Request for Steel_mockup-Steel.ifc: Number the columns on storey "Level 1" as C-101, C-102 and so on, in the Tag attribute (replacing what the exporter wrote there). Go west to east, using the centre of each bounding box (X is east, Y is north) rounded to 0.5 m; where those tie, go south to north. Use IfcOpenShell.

First a look at what the model holds.

```python
import ifcopenshell
import ifcopenshell.util.element
import ifcopenshell.util.placement

model = ifcopenshell.open("Steel_mockup-Steel.ifc")
print(model.schema)
storey = next(s for s in model.by_type("IfcBuildingStorey") if s.Name == "Level 1")
columns = [e for e in ifcopenshell.util.element.get_decomposition(storey) if e.is_a("IfcColumn")]
for e in sorted(columns, key=lambda e: e.id()):
    origin = ifcopenshell.util.placement.get_local_placement(e.ObjectPlacement)[:3, 3]
    print(e.id(), e.Tag, e.Name, origin.round(2) + 0.0, sep=" | ")
```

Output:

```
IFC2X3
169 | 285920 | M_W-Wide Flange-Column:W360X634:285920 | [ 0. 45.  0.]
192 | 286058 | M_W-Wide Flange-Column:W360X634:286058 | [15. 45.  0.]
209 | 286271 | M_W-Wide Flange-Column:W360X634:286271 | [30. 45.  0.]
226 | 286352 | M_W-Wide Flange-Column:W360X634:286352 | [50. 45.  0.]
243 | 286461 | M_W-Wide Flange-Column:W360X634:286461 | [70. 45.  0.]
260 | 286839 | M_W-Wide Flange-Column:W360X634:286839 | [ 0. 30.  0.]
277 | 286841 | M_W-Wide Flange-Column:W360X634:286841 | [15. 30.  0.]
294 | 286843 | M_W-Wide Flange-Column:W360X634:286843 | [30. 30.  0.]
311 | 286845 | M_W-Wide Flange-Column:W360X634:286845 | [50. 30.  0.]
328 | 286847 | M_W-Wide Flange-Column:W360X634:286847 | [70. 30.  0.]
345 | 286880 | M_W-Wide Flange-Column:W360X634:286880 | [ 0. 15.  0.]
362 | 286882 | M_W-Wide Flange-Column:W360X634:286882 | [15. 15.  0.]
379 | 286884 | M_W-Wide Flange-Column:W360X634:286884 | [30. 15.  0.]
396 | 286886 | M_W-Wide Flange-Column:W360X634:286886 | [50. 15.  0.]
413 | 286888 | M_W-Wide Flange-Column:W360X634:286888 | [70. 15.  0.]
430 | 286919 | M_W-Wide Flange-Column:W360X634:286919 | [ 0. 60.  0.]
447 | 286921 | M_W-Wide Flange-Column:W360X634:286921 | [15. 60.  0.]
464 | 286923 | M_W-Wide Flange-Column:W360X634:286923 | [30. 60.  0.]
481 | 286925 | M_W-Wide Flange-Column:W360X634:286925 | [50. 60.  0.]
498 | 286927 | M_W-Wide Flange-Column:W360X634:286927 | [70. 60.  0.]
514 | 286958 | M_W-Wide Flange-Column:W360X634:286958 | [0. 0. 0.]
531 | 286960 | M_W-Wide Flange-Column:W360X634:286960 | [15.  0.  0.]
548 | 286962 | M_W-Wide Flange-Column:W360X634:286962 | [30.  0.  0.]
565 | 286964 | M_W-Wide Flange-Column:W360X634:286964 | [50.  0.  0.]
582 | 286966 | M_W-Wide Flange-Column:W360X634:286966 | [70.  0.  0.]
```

```python
import ifcopenshell
import ifcopenshell.geom
import ifcopenshell.util.element
import ifcopenshell.util.shape

model = ifcopenshell.open("Steel_mockup-Steel.ifc")
settings = ifcopenshell.geom.settings()
settings.set("use-world-coords", True)


def centre(element):
    shape = ifcopenshell.geom.create_shape(settings, element)
    return ifcopenshell.util.shape.get_bbox_centroid(shape.geometry)


storey = next(s for s in model.by_type("IfcBuildingStorey") if s.Name == "Level 1")
columns = [e for e in ifcopenshell.util.element.get_decomposition(storey) if e.is_a("IfcColumn")]

# Insertion points can sit at a corner or the storey origin, so sort by the geometry (in metres).
centres = {e: centre(e) for e in columns}
columns.sort(key=lambda e: (round(centres[e][0] / 0.5), centres[e][1]))

for i, e in enumerate(columns, start=1):
    number = f"C-1{i:02d}"
    e.Tag = number
    print(e.id(), number)

model.write("Steel_mockup-Steel_v2.ifc")
```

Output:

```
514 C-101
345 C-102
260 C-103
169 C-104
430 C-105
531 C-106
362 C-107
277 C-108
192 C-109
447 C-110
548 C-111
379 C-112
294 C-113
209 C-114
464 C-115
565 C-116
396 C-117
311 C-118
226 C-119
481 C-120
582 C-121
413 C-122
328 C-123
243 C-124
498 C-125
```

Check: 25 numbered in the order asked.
